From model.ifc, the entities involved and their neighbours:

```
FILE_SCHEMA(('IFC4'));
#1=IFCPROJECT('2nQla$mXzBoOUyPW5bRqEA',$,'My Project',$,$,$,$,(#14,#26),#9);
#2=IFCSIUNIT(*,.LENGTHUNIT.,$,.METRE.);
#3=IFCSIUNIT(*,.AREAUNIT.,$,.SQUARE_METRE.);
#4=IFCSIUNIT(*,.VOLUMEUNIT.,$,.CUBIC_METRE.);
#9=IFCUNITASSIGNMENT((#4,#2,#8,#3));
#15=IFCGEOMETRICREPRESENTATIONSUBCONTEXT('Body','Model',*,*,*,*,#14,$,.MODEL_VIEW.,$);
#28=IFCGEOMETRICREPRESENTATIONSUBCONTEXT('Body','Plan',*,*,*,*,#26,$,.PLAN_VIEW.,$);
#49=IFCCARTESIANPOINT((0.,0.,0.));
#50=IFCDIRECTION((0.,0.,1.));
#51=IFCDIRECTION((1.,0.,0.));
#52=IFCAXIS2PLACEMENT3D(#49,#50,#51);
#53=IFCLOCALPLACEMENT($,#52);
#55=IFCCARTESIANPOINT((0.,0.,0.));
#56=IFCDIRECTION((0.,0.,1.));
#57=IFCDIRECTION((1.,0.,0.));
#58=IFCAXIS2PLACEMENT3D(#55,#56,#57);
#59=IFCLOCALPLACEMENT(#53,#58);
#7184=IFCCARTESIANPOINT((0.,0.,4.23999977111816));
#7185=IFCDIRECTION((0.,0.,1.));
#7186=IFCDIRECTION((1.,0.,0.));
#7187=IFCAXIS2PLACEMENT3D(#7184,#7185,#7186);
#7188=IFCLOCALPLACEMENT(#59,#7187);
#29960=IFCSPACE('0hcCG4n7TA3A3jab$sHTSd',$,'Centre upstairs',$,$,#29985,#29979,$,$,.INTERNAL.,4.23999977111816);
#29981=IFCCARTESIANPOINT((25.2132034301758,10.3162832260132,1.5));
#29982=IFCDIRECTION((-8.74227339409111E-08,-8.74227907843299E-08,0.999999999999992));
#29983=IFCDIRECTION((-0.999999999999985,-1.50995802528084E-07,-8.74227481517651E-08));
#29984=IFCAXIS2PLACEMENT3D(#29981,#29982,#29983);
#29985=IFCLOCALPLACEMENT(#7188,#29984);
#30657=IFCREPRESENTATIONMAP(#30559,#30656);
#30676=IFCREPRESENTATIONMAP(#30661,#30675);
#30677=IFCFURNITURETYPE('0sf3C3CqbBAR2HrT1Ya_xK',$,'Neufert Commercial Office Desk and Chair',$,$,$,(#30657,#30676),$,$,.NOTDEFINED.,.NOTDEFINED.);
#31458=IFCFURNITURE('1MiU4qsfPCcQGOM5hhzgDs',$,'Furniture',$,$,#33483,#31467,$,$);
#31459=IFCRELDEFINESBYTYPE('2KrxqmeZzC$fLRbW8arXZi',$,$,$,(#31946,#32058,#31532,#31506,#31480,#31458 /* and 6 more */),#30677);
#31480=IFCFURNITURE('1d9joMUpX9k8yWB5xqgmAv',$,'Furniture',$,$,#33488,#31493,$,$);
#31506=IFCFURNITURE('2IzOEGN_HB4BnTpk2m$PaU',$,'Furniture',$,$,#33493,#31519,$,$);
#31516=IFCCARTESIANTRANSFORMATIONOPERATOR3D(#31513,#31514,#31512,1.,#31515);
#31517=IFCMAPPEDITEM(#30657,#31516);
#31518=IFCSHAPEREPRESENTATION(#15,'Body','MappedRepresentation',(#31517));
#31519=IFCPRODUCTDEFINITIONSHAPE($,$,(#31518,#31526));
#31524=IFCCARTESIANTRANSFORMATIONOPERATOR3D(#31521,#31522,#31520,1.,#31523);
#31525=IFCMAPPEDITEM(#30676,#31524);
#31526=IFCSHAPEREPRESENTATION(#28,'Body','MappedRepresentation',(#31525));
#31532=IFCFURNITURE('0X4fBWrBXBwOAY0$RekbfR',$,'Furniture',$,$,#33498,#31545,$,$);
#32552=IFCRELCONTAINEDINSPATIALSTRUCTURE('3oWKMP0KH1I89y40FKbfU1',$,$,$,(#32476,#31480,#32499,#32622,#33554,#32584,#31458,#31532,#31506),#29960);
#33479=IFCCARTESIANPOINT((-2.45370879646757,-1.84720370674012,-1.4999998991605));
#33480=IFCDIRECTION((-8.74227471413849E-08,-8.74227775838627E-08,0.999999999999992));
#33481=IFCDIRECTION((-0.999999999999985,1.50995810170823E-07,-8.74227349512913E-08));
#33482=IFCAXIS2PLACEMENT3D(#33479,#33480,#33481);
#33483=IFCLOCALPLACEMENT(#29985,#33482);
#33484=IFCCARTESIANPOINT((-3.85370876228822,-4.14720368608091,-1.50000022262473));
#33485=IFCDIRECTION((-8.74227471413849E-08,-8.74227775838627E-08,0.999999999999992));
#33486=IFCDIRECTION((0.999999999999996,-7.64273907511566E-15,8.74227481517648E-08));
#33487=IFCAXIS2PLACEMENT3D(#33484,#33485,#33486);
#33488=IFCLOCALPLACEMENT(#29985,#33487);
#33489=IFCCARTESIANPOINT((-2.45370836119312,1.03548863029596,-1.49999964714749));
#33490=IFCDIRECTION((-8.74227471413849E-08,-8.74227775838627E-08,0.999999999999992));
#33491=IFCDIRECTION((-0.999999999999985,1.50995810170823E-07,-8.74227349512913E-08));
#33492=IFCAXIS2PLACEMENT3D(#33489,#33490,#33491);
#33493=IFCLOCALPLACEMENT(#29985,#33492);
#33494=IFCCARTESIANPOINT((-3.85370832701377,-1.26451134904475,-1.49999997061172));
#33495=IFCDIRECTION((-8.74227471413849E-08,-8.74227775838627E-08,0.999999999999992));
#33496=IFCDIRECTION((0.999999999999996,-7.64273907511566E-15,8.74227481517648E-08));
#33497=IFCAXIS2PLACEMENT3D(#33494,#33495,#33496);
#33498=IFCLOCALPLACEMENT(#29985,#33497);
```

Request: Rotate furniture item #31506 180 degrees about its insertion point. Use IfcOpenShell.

```python
import ifcopenshell
import ifcopenshell.api.geometry
import ifcopenshell.util.placement

model = ifcopenshell.open("model.ifc")

item = model.by_guid("2IzOEGN_HB4BnTpk2m$PaU")
matrix = ifcopenshell.util.placement.get_local_placement(item.ObjectPlacement)
matrix = matrix @ ifcopenshell.util.placement.rotation(180, "Z")
ifcopenshell.api.geometry.edit_object_placement(model, product=item, matrix=matrix, is_si=False)

print(ifcopenshell.util.placement.get_local_placement(item.ObjectPlacement).round(3) + 0.0)

model.write("model_v2.ifc")
```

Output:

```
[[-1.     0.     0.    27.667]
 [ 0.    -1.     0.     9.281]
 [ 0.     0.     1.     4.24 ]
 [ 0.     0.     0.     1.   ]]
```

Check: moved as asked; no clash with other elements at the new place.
